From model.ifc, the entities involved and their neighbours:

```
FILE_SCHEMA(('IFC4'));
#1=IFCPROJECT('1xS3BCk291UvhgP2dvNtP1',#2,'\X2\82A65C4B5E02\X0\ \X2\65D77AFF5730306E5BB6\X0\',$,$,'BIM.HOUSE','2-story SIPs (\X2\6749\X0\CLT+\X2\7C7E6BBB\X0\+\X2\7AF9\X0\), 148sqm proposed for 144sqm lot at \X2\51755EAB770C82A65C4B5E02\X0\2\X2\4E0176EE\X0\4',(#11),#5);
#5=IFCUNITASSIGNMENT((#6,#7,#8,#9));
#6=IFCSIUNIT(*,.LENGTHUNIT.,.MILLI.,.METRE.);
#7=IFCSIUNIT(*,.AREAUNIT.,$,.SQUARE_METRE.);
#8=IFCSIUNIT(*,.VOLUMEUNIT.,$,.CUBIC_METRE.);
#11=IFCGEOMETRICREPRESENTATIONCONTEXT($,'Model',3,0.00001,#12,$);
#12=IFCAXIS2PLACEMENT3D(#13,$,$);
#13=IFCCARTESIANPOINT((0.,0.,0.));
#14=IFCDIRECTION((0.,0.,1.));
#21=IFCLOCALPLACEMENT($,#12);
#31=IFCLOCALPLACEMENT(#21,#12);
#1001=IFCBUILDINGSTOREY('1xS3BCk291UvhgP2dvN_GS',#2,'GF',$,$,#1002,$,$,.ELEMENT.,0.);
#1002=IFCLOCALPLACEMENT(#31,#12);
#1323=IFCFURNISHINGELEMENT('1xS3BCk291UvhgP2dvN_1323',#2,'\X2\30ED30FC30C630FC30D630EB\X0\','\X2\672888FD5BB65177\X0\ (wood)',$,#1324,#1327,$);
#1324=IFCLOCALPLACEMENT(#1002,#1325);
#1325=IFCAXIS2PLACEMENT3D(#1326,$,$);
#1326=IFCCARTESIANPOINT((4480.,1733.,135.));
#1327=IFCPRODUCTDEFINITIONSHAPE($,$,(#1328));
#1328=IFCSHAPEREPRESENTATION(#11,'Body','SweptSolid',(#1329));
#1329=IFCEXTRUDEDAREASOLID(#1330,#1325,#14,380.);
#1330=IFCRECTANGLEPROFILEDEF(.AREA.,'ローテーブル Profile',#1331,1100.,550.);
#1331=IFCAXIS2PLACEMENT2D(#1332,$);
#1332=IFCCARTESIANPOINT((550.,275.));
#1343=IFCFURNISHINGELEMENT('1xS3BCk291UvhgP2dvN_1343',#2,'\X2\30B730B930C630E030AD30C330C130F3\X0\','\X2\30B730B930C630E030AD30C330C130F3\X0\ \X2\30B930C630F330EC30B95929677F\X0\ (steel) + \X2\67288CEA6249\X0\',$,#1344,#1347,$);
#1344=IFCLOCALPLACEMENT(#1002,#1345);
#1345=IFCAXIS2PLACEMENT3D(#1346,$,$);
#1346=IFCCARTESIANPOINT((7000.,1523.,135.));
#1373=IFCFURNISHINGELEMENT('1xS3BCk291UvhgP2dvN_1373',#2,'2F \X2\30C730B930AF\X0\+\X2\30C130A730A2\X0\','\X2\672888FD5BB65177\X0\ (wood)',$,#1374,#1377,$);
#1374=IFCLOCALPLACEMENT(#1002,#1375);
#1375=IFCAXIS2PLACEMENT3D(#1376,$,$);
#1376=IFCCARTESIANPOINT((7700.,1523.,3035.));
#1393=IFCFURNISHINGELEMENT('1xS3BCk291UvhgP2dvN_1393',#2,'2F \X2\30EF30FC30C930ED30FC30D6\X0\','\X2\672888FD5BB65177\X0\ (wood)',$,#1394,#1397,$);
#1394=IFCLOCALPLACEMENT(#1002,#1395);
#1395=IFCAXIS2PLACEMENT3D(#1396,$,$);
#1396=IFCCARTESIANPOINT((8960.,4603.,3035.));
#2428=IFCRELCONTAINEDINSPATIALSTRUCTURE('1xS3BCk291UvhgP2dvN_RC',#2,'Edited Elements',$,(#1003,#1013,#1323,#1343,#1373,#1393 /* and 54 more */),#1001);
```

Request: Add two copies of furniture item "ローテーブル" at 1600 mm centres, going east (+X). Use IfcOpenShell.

```python
import numpy as np
import ifcopenshell
import ifcopenshell.api.geometry
import ifcopenshell.api.root
import ifcopenshell.util.element
import ifcopenshell.util.placement
import ifcopenshell.util.unit

model = ifcopenshell.open("model.ifc")
unit_scale = ifcopenshell.util.unit.calculate_unit_scale(model)


def reuse_history(source, copy):
    """copy_class also copies each property set's owner history, people and application; keep the originals."""
    for rel in copy.IsDefinedBy:
        if rel.is_a("IfcRelDefinesByProperties") and (history := rel.RelatingPropertyDefinition.OwnerHistory):
            rel.RelatingPropertyDefinition.OwnerHistory = source.OwnerHistory
            ifcopenshell.util.element.remove_deep2(model, history)


source = model.by_id(1323)
base = ifcopenshell.util.placement.get_local_placement(source.ObjectPlacement)
step = np.array([1.0, 0.0, 0.0]) * 1.6 / unit_scale

for i in range(1, 3):
    copy = ifcopenshell.api.root.copy_class(model, product=source)
    copy.Representation = ifcopenshell.util.element.copy_deep(
        model, source.Representation, exclude=["IfcGeometricRepresentationContext", "IfcRepresentationMap"]
    )
    reuse_history(source, copy)
    matrix = base.copy()
    matrix[:3, 3] += i * step
    print("added at", matrix[:3, 3].round(3) + 0.0)
    ifcopenshell.api.geometry.edit_object_placement(model, product=copy, matrix=matrix, is_si=False)

model.write("model_v2.ifc")
```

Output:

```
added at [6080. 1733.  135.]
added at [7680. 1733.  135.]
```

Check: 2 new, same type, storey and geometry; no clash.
